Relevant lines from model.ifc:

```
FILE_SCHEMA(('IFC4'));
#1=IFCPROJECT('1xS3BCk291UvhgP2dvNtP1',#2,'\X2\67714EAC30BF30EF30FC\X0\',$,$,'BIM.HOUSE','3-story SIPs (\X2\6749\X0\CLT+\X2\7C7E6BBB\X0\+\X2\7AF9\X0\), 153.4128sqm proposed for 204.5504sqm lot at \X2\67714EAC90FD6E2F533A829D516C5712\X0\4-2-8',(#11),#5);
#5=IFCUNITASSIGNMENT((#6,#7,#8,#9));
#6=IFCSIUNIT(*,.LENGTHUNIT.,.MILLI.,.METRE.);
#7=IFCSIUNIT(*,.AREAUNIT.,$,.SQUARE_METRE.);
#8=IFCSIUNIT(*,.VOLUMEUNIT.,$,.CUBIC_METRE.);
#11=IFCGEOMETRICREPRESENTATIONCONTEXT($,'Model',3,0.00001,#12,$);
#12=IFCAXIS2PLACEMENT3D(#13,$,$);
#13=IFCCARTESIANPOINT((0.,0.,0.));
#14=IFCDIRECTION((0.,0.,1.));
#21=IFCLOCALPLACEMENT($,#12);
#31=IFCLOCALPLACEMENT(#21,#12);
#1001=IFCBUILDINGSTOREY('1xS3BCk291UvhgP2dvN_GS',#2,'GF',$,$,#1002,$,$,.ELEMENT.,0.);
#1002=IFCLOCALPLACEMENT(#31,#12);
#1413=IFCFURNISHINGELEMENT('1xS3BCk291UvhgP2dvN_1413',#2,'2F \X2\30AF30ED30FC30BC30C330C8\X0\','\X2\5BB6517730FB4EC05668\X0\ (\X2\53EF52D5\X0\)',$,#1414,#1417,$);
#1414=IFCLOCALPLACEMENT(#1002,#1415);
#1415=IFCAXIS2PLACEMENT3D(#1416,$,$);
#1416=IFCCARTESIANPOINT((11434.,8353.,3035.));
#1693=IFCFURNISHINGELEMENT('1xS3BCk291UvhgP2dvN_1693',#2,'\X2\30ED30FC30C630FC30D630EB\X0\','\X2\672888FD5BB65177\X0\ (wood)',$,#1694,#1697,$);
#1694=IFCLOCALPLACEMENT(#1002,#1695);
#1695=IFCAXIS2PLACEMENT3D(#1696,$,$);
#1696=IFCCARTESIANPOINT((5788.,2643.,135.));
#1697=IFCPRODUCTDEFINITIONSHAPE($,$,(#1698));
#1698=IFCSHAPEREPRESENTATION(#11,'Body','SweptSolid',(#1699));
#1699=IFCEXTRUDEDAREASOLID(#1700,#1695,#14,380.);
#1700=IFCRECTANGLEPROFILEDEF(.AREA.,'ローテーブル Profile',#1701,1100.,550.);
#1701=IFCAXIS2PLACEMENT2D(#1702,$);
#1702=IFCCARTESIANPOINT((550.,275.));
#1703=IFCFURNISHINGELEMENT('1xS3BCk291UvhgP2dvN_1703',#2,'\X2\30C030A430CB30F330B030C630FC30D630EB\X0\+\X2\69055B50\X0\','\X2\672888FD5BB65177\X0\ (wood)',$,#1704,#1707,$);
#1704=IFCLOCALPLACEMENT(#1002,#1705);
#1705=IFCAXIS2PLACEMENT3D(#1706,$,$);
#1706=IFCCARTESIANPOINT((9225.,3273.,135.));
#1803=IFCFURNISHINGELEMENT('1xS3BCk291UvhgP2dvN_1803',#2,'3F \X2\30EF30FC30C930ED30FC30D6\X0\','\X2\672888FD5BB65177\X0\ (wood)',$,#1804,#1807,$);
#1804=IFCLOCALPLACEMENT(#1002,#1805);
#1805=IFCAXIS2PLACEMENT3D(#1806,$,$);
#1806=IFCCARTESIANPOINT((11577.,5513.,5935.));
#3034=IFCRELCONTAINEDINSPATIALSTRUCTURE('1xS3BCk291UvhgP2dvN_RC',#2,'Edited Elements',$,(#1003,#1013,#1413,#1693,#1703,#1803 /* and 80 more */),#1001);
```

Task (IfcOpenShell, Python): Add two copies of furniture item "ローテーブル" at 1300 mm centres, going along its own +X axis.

```python
import ifcopenshell
import ifcopenshell.api.geometry
import ifcopenshell.api.root
import ifcopenshell.util.element
import ifcopenshell.util.placement
import ifcopenshell.util.unit

model = ifcopenshell.open("model.ifc")
unit_scale = ifcopenshell.util.unit.calculate_unit_scale(model)


def reuse_history(source, copy):
    """copy_class also copies each property set's owner history, people and application; keep the originals."""
    for rel in copy.IsDefinedBy:
        if rel.is_a("IfcRelDefinesByProperties") and (history := rel.RelatingPropertyDefinition.OwnerHistory):
            rel.RelatingPropertyDefinition.OwnerHistory = source.OwnerHistory
            ifcopenshell.util.element.remove_deep2(model, history)


source = model.by_guid("1xS3BCk291UvhgP2dvN_1693")
base = ifcopenshell.util.placement.get_local_placement(source.ObjectPlacement)
step = base[:3, 0] * 1.3 / unit_scale

for i in range(1, 3):
    copy = ifcopenshell.api.root.copy_class(model, product=source)
    copy.Representation = ifcopenshell.util.element.copy_deep(
        model, source.Representation, exclude=["IfcGeometricRepresentationContext", "IfcRepresentationMap"]
    )
    reuse_history(source, copy)
    matrix = base.copy()
    matrix[:3, 3] += i * step
    print("added at", matrix[:3, 3].round(3) + 0.0)
    ifcopenshell.api.geometry.edit_object_placement(model, product=copy, matrix=matrix, is_si=False)

model.write("model_v2.ifc")
```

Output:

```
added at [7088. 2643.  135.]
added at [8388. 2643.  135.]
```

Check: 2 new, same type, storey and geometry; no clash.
